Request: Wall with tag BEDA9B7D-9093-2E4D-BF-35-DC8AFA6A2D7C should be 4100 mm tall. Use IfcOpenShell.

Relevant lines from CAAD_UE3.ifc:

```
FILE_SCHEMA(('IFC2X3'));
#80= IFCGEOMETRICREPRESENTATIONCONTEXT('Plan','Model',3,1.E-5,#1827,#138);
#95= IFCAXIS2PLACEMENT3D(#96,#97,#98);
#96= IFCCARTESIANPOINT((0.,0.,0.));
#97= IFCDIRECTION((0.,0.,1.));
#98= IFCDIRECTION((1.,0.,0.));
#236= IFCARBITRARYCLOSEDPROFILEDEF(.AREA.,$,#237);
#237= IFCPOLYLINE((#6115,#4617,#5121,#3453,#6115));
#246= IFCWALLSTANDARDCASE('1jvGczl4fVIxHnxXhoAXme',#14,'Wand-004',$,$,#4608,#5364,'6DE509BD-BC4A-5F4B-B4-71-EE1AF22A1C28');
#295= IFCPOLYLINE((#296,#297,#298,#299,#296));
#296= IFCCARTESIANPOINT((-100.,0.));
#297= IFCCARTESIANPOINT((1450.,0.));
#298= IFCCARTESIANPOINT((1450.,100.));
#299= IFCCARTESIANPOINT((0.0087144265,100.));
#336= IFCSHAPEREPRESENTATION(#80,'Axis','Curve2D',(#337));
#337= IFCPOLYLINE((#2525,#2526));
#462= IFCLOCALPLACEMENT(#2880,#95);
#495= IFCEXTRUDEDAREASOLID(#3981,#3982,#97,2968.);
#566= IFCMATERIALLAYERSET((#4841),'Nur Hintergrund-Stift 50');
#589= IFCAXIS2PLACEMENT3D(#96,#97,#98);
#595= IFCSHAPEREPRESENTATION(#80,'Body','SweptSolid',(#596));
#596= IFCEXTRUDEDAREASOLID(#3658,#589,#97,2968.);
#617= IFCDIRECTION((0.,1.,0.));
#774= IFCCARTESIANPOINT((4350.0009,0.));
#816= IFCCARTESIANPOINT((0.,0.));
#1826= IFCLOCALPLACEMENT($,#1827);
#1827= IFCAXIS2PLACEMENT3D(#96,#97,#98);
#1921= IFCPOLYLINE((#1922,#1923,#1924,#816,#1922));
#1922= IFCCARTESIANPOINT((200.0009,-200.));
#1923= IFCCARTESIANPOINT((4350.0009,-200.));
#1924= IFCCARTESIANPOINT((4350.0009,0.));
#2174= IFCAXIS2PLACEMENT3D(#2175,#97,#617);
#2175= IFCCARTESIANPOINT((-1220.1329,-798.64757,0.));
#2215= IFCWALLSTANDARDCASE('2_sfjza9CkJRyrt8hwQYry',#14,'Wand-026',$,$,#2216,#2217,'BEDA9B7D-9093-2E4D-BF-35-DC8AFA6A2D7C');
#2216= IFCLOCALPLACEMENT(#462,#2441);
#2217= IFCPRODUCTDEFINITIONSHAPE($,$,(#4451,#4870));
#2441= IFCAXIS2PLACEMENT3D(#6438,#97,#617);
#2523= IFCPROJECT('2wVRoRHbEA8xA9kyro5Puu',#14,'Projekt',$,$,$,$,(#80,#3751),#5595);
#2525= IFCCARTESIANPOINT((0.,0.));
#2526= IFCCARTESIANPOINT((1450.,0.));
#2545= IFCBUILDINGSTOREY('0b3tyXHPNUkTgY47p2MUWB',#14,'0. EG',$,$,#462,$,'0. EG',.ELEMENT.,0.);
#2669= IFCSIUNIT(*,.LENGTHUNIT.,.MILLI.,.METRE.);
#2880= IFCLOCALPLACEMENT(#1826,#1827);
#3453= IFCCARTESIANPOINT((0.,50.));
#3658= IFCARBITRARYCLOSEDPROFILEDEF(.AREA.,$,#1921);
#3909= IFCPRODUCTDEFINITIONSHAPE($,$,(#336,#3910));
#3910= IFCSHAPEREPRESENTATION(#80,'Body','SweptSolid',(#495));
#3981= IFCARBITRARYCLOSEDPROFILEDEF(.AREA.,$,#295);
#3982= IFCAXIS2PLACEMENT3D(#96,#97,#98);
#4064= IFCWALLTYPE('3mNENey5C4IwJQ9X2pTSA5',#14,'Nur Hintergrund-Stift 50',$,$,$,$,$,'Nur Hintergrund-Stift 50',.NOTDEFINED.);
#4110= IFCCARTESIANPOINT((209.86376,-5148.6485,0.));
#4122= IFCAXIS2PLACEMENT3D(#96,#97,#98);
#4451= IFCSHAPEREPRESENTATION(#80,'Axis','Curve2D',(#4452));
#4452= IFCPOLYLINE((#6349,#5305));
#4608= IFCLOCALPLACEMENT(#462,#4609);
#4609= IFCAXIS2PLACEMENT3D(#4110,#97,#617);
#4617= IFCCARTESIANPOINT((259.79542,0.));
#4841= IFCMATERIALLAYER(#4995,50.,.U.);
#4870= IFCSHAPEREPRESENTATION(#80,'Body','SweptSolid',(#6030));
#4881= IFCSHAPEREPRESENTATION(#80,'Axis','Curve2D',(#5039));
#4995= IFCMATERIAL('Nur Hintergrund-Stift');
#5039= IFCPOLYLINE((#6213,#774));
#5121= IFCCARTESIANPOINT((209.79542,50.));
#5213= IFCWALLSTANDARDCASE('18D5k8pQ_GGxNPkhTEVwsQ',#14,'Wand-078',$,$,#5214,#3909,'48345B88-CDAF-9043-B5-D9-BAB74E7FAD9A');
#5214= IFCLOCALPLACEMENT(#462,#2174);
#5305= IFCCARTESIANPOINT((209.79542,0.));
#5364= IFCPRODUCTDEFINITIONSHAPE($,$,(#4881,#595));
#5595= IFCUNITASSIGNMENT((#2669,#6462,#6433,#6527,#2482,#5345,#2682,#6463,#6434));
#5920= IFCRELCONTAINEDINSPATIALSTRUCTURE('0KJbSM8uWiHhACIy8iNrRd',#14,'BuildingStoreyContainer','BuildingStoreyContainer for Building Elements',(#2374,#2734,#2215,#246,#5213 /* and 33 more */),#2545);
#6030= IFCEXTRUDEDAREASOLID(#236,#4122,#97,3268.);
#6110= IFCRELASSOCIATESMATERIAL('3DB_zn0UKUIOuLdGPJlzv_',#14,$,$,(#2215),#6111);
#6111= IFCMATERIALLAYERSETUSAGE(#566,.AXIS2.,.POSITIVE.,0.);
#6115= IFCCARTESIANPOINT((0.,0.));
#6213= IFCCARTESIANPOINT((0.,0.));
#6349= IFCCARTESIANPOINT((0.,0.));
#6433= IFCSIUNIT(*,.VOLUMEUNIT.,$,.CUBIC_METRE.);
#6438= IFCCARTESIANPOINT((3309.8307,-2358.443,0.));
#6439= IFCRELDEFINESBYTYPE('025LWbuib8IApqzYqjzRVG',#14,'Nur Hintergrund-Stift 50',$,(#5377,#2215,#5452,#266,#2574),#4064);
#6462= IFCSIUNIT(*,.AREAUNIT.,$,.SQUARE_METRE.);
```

```python
import ifcopenshell
import ifcopenshell.geom
import ifcopenshell.util.shape
import ifcopenshell.util.unit

model = ifcopenshell.open("CAAD_UE3.ifc")
unit_scale = ifcopenshell.util.unit.calculate_unit_scale(model)
settings = ifcopenshell.geom.settings()


def volume(element):
    """Net volume in cubic metres, openings subtracted."""
    shape = ifcopenshell.geom.create_shape(settings, element)
    return ifcopenshell.util.shape.get_volume(shape.geometry)


wall = model.by_guid("2_sfjza9CkJRyrt8hwQYry")
before = volume(wall)

body = next(r for r in wall.Representation.Representations if r.RepresentationIdentifier == "Body")
solid = body.Items[0]
old_height = solid.Depth
solid.Depth = 4.1 / unit_scale
after = volume(wall)

print(f"height {old_height:g} -> {solid.Depth:g}, volume {before:.3f} -> {after:.3f} m3")

model.write("CAAD_UE3_v2.ifc")
```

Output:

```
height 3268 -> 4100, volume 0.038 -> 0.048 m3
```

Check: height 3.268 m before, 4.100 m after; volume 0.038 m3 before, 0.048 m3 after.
